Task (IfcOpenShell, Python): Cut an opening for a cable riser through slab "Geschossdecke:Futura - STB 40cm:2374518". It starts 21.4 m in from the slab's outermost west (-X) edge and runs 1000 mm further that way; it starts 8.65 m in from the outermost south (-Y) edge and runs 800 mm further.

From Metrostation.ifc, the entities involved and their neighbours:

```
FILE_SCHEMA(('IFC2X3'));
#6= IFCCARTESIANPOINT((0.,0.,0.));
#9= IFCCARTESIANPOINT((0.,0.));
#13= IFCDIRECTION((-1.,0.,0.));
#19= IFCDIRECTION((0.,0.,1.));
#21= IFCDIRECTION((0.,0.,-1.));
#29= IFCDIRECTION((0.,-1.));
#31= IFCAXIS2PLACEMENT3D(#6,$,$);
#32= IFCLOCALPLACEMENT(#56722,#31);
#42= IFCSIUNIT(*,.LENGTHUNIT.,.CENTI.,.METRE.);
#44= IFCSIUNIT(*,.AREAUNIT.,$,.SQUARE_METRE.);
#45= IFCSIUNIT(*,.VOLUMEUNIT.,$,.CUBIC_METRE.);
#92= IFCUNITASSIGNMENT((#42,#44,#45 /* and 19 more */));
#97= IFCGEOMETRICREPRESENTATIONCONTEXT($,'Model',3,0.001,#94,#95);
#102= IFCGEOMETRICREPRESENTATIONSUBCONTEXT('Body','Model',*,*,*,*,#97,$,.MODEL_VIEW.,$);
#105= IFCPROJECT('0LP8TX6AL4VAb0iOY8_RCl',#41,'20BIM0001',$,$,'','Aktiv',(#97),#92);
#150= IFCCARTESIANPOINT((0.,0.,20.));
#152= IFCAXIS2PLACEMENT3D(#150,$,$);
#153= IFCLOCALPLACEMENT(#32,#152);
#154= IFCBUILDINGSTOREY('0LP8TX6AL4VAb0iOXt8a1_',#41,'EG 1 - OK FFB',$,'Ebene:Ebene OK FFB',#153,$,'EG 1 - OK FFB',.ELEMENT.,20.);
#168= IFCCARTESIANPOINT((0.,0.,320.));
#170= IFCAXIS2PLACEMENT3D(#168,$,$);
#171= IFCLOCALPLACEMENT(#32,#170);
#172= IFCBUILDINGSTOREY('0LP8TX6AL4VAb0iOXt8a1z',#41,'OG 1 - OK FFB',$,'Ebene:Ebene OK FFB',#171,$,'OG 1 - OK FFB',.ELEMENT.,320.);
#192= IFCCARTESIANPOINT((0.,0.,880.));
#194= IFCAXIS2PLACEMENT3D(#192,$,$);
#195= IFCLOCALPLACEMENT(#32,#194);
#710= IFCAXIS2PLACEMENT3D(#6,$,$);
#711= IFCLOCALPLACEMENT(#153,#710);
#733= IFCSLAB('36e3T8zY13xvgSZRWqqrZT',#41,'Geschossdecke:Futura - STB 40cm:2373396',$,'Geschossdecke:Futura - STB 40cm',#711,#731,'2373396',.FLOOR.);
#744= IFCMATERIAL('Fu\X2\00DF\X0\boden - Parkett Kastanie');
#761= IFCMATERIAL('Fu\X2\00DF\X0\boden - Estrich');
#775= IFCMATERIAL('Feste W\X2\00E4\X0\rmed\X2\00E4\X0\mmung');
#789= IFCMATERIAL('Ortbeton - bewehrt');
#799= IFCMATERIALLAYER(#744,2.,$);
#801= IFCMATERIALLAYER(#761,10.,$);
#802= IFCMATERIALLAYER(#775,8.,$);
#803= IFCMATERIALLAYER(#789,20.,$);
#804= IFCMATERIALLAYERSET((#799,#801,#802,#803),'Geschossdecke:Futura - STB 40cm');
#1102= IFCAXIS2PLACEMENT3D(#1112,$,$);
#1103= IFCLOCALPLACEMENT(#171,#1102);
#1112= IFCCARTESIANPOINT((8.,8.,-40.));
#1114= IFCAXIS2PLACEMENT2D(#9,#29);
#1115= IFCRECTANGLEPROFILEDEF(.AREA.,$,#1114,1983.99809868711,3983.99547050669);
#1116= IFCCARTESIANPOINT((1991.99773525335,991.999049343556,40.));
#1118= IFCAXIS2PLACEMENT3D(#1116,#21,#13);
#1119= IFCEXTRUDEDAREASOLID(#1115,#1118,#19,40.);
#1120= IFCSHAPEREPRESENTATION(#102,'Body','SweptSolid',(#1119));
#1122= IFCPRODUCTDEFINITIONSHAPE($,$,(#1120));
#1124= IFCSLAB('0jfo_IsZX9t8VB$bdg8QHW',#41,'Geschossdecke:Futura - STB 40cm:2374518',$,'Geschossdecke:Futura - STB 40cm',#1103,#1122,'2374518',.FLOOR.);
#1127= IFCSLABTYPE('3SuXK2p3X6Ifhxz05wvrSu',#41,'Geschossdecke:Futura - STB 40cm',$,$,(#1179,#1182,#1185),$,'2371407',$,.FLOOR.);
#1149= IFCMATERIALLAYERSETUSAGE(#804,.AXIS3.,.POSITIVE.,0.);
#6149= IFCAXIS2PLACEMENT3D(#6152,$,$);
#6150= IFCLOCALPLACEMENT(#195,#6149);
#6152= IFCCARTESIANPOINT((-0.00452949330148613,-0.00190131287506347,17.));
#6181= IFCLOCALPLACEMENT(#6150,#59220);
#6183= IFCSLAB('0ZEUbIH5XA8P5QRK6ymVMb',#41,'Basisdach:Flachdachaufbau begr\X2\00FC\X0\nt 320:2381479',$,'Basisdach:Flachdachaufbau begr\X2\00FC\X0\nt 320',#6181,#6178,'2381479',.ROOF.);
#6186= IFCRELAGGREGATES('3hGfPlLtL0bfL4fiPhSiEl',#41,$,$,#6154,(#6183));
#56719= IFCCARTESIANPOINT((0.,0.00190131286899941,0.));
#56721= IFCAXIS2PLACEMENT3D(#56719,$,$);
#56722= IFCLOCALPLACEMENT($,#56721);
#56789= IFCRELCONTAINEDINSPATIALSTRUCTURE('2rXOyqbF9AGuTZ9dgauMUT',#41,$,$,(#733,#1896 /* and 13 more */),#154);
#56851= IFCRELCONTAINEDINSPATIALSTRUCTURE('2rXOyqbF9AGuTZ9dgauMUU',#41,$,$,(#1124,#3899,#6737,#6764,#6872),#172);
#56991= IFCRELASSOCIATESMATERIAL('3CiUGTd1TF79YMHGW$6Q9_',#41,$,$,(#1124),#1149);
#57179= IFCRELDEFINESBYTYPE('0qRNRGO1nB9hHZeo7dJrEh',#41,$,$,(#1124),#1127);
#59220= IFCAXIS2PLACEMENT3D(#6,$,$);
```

```python
import numpy as np
import ifcopenshell
import ifcopenshell.api.feature
import ifcopenshell.api.geometry
import ifcopenshell.api.root
import ifcopenshell.geom
import ifcopenshell.util.placement
import ifcopenshell.util.representation
import ifcopenshell.util.shape
import ifcopenshell.util.unit

model = ifcopenshell.open("Metrostation.ifc")
unit_scale = ifcopenshell.util.unit.calculate_unit_scale(model)
settings = ifcopenshell.geom.settings()


def volume(element):
    """Net volume in cubic metres, openings subtracted."""
    shape = ifcopenshell.geom.create_shape(settings, element)
    return ifcopenshell.util.shape.get_volume(shape.geometry)


slab = model.by_guid("0jfo_IsZX9t8VB$bdg8QHW")
before = volume(slab)

# Extent in the slab's own axes, in metres. The edges named are its -X and -Y sides.
slab_shape = ifcopenshell.geom.create_shape(settings, slab)
vertices = ifcopenshell.util.shape.get_vertices(slab_shape.geometry)
x_min, y_min, bottom = vertices.min(axis=0)
top = vertices[:, 2].max()

opening = ifcopenshell.api.root.create_entity(model, ifc_class="IfcOpeningElement", name="Cable riser opening")
context = ifcopenshell.util.representation.get_context(model, "Model", "Body", "MODEL_VIEW")
width, depth = 1, 0.8
outline = [(0.0, 0.0), (width, 0.0), (width, depth), (0.0, depth), (0.0, 0.0)]
# Overshoot both faces by 50 mm so the cut is clean.
shape = ifcopenshell.api.geometry.add_slab_representation(
    model, context=context, depth=top - bottom + 0.1, polyline=outline
)
ifcopenshell.api.geometry.assign_representation(model, product=opening, representation=shape)

matrix = ifcopenshell.util.placement.get_local_placement(slab.ObjectPlacement)
matrix[:, 3] = matrix @ np.append(np.array([x_min + 21.4, y_min + 8.65, bottom - 0.05]) / unit_scale, 1.0)
ifcopenshell.api.geometry.edit_object_placement(model, product=opening, matrix=matrix, is_si=False)
ifcopenshell.api.feature.add_feature(model, feature=opening, element=slab)

after = volume(slab)

print(f"slab volume {before:.3f} -> {after:.3f} m3")

model.write("Metrostation-out.ifc")
```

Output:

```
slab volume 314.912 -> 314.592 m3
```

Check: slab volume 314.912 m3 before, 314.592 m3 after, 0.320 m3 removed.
